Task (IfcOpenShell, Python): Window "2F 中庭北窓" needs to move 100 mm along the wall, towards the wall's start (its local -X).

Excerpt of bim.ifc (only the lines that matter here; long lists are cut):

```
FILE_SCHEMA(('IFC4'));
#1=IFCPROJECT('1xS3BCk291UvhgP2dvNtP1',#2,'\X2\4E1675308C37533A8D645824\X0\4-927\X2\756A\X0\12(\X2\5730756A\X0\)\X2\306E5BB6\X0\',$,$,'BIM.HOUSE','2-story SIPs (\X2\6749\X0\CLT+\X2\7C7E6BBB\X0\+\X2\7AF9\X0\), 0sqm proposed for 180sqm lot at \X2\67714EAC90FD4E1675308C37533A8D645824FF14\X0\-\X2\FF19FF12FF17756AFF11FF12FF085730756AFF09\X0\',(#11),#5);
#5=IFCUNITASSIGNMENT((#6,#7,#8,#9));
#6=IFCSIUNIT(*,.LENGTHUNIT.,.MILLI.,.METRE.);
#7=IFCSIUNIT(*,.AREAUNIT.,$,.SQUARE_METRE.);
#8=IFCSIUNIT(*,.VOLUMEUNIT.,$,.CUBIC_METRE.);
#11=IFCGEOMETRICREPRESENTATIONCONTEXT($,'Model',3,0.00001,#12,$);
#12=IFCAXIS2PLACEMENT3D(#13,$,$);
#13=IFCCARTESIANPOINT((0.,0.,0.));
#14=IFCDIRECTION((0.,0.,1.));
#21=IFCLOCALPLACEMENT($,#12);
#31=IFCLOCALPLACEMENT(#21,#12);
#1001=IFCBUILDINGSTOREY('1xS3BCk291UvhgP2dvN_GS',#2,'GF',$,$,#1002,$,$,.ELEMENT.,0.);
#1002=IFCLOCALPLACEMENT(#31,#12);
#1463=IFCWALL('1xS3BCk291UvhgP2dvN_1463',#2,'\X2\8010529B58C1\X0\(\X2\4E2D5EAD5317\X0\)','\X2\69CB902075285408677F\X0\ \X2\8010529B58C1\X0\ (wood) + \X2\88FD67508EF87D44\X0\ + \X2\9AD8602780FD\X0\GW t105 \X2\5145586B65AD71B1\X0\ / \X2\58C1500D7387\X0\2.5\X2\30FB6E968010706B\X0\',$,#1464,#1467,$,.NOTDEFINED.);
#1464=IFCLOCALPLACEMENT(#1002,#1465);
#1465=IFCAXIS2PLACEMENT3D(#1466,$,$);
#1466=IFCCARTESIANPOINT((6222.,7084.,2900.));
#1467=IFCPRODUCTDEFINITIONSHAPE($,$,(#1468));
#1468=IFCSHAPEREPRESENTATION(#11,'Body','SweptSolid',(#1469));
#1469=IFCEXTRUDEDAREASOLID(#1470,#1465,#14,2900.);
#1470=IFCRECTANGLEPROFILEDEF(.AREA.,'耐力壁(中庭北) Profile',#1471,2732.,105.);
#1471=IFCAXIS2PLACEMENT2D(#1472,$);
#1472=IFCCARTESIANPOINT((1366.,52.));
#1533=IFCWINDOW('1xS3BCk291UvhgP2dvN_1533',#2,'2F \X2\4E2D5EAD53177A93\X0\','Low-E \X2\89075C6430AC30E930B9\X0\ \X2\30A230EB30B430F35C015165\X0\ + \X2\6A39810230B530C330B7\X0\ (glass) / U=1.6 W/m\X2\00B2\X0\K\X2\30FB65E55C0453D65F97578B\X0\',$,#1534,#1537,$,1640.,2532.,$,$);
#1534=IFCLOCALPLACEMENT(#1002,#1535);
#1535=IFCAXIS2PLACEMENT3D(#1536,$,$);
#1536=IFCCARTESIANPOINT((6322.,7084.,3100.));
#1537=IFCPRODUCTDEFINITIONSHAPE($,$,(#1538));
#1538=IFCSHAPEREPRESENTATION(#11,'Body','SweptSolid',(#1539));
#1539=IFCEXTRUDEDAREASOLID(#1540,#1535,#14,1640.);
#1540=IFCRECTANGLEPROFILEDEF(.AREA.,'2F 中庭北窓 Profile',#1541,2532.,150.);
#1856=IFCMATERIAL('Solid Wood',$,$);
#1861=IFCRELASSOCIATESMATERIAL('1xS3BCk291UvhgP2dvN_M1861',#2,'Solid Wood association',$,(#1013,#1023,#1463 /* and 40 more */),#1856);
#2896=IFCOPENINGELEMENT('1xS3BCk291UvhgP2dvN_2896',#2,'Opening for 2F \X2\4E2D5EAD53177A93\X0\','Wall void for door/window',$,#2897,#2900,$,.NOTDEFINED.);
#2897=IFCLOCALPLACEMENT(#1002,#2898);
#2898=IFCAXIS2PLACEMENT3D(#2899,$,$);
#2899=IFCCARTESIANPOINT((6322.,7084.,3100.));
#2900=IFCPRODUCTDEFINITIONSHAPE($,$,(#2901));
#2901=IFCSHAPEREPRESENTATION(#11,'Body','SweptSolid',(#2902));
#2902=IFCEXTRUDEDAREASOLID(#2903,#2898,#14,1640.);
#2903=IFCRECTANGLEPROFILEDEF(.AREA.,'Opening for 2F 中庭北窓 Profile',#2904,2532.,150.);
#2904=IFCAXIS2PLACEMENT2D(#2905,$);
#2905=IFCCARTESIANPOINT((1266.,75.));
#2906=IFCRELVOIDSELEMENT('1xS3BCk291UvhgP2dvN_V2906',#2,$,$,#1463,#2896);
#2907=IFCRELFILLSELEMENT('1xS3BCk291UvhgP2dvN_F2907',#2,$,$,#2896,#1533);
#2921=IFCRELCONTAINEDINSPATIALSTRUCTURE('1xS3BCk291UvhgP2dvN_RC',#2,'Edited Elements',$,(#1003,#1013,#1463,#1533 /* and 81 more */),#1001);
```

```python
import ifcopenshell
import ifcopenshell.api.geometry
import ifcopenshell.util.placement
import ifcopenshell.util.unit

model = ifcopenshell.open("bim.ifc")
unit_scale = ifcopenshell.util.unit.calculate_unit_scale(model)

window = model.by_guid("1xS3BCk291UvhgP2dvN_1533")
opening = window.FillsVoids[0].RelatingOpeningElement
wall = opening.VoidsElements[0].RelatingBuildingElement

wall_matrix = ifcopenshell.util.placement.get_local_placement(wall.ObjectPlacement)
shift = wall_matrix[:3, 0] * -0.1 / unit_scale
before = ifcopenshell.util.placement.get_local_placement(window.ObjectPlacement)[:3, 3].copy()

# The window is not placed relative to its opening, so move both.
for product in (opening, window):
    matrix = ifcopenshell.util.placement.get_local_placement(product.ObjectPlacement)
    matrix[:3, 3] += shift
    ifcopenshell.api.geometry.edit_object_placement(model, product=product, matrix=matrix, is_si=False)

after = ifcopenshell.util.placement.get_local_placement(window.ObjectPlacement)[:3, 3]
print("window moved by", (after - before).round(3) + 0.0)

model.write("bim_updated.ifc")
```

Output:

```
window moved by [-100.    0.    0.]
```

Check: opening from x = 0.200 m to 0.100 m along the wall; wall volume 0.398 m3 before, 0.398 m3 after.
